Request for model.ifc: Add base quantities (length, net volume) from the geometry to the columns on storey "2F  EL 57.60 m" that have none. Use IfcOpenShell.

First a look at what the model holds.

```python
import ifcopenshell
import ifcopenshell.util.element
import ifcopenshell.util.unit

model = ifcopenshell.open("model.ifc")
print(model.schema)
for unit_type in ("LENGTHUNIT", "AREAUNIT", "VOLUMEUNIT"):
    print(unit_type, ifcopenshell.util.unit.calculate_unit_scale(model, unit_type))
storey = next(s for s in model.by_type("IfcBuildingStorey") if s.Name == "2F  EL 57.60 m")
columns = [e for e in ifcopenshell.util.element.get_decomposition(storey) if e.is_a("IfcColumn")]
for e in sorted(columns, key=lambda e: e.id()):
    print(e.id(), e.is_a(), e.Name, list(ifcopenshell.util.element.get_psets(e, qtos_only=True)), sep=" | ")
```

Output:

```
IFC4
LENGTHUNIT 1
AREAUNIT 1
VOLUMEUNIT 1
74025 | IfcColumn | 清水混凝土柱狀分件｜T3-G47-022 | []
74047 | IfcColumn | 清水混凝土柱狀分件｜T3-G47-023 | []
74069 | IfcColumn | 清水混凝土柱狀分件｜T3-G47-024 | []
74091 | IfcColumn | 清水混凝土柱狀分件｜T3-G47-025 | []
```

```python
import ifcopenshell
import ifcopenshell.api.pset
import ifcopenshell.geom
import ifcopenshell.util.element
import ifcopenshell.util.shape
import ifcopenshell.util.unit

model = ifcopenshell.open("model.ifc")
unit_scale = ifcopenshell.util.unit.calculate_unit_scale(model)
volume_scale = ifcopenshell.util.unit.calculate_unit_scale(model, "VOLUMEUNIT")
settings = ifcopenshell.geom.settings()

storey = next(s for s in model.by_type("IfcBuildingStorey") if s.Name == "2F  EL 57.60 m")
columns = [e for e in ifcopenshell.util.element.get_decomposition(storey) if e.is_a("IfcColumn")]

for e in sorted(columns, key=lambda e: e.id()):
    if ifcopenshell.util.element.get_psets(e, qtos_only=True, should_inherit=False):
        continue
    # Geometry comes back in metres, in the element's own axes.
    shape = ifcopenshell.geom.create_shape(settings, e)
    values = {
        "Length": ifcopenshell.util.shape.get_z(shape.geometry) / unit_scale,
        "NetVolume": ifcopenshell.util.shape.get_volume(shape.geometry) / volume_scale,
    }
    qto = ifcopenshell.api.pset.add_qto(model, product=e, name="Qto_ColumnBaseQuantities")
    ifcopenshell.api.pset.edit_qto(model, qto=qto, properties=values)
    print(e.id(), {k: round(v, 3) for k, v in values.items()})

model.write("model-out.ifc")
```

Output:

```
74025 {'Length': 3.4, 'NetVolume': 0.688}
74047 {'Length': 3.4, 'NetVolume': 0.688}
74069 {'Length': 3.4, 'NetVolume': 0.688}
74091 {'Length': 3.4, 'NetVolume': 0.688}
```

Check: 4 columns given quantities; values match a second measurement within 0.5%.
